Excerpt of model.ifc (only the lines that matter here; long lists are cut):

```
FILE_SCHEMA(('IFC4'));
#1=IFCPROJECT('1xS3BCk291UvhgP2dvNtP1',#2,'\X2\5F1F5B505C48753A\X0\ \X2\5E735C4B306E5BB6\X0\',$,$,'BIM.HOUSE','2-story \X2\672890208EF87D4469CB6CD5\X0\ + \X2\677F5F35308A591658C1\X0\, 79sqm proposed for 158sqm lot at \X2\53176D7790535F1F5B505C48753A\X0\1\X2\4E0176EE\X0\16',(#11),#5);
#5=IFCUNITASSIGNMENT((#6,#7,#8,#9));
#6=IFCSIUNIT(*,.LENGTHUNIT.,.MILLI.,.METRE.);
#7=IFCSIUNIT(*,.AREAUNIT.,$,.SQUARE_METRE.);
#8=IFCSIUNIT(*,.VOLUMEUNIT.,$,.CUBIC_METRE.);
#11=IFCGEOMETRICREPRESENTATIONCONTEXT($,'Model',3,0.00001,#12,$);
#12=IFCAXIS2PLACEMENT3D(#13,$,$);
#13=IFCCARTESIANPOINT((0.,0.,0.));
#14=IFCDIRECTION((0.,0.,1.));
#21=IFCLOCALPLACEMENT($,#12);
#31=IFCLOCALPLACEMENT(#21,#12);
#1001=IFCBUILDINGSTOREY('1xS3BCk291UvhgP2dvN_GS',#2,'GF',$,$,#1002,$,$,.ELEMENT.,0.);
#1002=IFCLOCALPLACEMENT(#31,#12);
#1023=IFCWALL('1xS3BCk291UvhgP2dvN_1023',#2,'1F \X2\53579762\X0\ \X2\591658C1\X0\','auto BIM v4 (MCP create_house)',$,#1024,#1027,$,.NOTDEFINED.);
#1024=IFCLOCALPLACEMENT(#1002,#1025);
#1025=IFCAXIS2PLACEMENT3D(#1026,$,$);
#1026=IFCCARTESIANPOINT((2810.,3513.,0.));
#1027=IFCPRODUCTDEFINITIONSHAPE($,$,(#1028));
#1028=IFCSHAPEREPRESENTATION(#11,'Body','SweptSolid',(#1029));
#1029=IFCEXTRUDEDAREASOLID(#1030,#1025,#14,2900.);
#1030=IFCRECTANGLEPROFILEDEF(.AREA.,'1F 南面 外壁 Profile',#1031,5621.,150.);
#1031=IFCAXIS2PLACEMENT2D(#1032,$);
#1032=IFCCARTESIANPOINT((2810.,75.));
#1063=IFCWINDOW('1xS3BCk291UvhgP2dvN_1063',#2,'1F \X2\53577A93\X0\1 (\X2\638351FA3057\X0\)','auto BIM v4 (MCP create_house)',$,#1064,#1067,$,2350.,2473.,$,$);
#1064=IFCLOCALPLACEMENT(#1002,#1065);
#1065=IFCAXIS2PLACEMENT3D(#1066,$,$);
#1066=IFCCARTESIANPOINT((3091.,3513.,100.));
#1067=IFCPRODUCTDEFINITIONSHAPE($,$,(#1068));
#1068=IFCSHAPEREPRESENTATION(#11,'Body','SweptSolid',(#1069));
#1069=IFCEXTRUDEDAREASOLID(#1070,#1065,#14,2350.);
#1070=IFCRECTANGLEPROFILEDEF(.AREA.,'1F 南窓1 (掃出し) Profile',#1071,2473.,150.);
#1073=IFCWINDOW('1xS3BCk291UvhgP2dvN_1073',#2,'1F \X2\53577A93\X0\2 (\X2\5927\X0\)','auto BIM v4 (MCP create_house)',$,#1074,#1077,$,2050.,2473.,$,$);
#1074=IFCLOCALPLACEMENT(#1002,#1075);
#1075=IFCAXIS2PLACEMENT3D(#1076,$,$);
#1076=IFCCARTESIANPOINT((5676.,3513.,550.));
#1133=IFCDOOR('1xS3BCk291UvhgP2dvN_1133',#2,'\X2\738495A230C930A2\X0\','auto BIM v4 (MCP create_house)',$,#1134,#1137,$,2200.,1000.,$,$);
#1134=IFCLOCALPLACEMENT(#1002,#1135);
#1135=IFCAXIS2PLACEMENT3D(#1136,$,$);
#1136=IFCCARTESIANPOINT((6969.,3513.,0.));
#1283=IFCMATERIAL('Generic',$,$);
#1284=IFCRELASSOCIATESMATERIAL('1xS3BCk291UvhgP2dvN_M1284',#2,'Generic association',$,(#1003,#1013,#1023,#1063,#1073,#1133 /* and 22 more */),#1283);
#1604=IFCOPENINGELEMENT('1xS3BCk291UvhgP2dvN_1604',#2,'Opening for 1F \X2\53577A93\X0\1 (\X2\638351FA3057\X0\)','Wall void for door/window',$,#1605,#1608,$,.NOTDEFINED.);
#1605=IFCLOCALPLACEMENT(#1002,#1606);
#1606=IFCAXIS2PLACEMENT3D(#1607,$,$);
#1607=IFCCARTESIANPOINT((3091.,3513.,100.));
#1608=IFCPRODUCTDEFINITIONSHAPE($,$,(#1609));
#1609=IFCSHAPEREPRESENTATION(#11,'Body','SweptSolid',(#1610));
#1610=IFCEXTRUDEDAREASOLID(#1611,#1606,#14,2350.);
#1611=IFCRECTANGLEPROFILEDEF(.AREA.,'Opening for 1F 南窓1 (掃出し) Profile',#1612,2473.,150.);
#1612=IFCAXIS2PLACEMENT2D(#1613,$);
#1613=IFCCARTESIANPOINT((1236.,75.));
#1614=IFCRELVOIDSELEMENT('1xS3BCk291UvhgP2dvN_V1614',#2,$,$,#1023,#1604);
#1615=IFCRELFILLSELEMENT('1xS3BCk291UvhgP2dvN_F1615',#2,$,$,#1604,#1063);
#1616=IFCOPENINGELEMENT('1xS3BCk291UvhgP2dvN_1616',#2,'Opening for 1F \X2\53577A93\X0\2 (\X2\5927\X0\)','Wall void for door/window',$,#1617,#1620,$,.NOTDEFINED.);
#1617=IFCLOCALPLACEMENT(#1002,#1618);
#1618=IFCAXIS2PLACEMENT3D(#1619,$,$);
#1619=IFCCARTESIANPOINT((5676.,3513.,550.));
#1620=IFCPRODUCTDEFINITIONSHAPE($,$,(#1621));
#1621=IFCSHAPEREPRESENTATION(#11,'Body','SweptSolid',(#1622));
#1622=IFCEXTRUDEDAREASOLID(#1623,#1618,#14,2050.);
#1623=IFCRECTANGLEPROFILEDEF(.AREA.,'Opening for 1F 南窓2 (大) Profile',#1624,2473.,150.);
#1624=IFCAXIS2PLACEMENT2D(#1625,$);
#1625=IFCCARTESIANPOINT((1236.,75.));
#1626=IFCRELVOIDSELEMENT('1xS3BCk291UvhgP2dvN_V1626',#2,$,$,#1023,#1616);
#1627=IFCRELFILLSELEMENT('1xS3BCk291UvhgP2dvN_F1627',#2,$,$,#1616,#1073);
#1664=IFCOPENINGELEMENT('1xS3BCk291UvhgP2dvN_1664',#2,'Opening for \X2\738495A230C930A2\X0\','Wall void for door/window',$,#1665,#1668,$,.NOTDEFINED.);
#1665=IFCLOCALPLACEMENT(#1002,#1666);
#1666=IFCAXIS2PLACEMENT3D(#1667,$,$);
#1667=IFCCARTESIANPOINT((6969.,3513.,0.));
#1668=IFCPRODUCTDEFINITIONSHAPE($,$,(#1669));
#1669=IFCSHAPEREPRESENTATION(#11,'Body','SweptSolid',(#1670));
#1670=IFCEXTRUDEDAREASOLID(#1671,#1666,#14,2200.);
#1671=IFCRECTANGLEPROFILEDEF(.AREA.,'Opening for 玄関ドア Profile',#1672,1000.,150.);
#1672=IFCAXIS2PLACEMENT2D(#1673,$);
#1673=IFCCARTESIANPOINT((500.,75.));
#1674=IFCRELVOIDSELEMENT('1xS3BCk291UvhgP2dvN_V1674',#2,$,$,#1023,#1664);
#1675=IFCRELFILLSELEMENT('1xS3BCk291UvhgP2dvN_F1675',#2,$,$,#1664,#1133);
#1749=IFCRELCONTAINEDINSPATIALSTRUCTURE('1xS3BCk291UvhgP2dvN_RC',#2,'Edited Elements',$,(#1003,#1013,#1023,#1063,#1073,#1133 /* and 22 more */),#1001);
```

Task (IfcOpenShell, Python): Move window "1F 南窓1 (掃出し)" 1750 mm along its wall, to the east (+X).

```python
import ifcopenshell
import ifcopenshell.api.geometry
import ifcopenshell.util.placement
import ifcopenshell.util.unit

model = ifcopenshell.open("model.ifc")
unit_scale = ifcopenshell.util.unit.calculate_unit_scale(model)

window = model.by_id(1063)
opening = window.FillsVoids[0].RelatingOpeningElement
wall = opening.VoidsElements[0].RelatingBuildingElement

wall_matrix = ifcopenshell.util.placement.get_local_placement(wall.ObjectPlacement)
shift = wall_matrix[:3, 0] * 1.75 / unit_scale
before = ifcopenshell.util.placement.get_local_placement(window.ObjectPlacement)[:3, 3].copy()

# The window is not placed relative to its opening, so move both.
for product in (opening, window):
    matrix = ifcopenshell.util.placement.get_local_placement(product.ObjectPlacement)
    matrix[:3, 3] += shift
    ifcopenshell.api.geometry.edit_object_placement(model, product=product, matrix=matrix, is_si=False)

after = ifcopenshell.util.placement.get_local_placement(window.ObjectPlacement)[:3, 3]
print("window moved by", (after - before).round(3) + 0.0)

model.write("model-out.ifc")
```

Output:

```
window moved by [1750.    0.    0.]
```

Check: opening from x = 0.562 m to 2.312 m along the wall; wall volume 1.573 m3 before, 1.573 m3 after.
